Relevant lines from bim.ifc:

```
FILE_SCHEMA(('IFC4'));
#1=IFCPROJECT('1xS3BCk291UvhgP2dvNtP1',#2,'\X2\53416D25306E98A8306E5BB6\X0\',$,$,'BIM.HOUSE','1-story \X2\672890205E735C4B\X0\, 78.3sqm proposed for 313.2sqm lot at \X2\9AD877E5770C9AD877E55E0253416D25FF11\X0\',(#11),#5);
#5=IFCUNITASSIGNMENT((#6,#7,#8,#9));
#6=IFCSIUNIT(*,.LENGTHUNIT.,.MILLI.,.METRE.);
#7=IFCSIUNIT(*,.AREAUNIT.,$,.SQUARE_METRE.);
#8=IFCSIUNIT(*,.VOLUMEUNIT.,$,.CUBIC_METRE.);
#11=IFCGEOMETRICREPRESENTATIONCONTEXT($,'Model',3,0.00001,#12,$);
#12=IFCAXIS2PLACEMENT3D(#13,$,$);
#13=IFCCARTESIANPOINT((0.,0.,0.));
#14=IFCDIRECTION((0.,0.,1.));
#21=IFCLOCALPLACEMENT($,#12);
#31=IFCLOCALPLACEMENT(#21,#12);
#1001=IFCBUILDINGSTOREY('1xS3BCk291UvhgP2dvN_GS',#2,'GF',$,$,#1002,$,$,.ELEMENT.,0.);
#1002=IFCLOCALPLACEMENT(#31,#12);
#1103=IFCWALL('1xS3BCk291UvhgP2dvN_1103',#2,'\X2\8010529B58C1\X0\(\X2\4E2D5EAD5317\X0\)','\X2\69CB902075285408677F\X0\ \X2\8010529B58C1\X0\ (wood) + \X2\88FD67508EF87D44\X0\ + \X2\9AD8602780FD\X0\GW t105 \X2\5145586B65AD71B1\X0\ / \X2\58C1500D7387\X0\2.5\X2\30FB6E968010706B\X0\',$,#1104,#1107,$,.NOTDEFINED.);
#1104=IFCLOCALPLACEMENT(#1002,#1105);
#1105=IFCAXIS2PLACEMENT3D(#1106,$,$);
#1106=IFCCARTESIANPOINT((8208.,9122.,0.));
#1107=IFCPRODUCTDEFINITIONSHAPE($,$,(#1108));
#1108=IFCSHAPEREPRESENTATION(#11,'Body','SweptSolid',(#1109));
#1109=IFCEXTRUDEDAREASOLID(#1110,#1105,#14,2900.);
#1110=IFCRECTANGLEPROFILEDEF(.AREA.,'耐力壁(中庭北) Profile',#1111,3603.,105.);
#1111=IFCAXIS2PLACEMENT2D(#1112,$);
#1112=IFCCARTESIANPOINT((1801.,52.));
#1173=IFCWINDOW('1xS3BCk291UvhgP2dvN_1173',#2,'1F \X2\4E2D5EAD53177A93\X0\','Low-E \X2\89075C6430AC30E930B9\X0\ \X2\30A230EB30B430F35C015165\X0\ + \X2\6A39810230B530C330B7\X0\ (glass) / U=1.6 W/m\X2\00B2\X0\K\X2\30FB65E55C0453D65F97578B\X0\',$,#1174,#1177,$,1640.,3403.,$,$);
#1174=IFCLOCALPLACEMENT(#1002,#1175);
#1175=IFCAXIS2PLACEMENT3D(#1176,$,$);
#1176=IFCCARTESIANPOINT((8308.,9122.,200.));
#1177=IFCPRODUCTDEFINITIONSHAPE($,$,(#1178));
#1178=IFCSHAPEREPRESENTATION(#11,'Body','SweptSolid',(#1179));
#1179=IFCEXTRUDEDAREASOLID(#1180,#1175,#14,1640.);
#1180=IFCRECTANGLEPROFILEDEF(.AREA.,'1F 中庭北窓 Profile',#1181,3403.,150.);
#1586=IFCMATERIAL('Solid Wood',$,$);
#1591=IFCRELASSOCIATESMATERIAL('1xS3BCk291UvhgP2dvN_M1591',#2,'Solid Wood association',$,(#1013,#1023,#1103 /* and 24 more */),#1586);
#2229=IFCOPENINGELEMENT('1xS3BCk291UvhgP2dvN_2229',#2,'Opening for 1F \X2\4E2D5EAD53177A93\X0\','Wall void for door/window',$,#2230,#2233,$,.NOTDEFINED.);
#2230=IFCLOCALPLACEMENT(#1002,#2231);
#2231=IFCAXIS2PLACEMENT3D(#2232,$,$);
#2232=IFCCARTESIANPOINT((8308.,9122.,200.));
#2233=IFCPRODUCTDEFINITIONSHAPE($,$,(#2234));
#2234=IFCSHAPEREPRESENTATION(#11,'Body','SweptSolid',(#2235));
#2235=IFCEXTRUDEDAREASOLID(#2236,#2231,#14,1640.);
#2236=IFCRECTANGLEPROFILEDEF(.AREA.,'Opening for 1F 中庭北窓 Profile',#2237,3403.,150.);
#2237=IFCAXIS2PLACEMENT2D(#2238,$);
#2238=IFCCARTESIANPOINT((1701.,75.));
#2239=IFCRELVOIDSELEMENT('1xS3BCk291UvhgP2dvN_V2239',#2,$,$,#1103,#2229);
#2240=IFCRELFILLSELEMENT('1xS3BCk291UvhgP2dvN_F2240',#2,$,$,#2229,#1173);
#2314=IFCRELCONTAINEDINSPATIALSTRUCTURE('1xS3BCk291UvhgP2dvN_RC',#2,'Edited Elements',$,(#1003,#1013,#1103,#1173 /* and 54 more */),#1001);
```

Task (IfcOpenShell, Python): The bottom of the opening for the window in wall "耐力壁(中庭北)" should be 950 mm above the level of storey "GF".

```python
import numpy as np
import ifcopenshell
import ifcopenshell.api.geometry
import ifcopenshell.geom
import ifcopenshell.util.element
import ifcopenshell.util.placement
import ifcopenshell.util.shape
import ifcopenshell.util.unit

model = ifcopenshell.open("bim.ifc")
unit_scale = ifcopenshell.util.unit.calculate_unit_scale(model)

window = model.by_guid("1xS3BCk291UvhgP2dvN_1173")
opening = window.FillsVoids[0].RelatingOpeningElement
storey = ifcopenshell.util.element.get_container(window, ifc_class="IfcBuildingStorey")
level = ifcopenshell.util.placement.get_local_placement(storey.ObjectPlacement)[2, 3]

# The opening's origin need not be at the sill, so measure its lowest point.
shape = ifcopenshell.geom.create_shape(ifcopenshell.geom.settings(), opening)
bottom = ifcopenshell.util.shape.get_shape_bottom_elevation(shape, shape.geometry) / unit_scale
dz = level + 0.95 / unit_scale - bottom

shift = np.array([0.0, 0.0, dz])
# The window is not placed relative to its opening, so move both.
for product in (opening, window):
    matrix = ifcopenshell.util.placement.get_local_placement(product.ObjectPlacement)
    matrix[:3, 3] += shift
    ifcopenshell.api.geometry.edit_object_placement(model, product=product, matrix=matrix, is_si=False)

print(f"moved by {dz * unit_scale:+.3f} m")

model.write("bim_edited.ifc")
```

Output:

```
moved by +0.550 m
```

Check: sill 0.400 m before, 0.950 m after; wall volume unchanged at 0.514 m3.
